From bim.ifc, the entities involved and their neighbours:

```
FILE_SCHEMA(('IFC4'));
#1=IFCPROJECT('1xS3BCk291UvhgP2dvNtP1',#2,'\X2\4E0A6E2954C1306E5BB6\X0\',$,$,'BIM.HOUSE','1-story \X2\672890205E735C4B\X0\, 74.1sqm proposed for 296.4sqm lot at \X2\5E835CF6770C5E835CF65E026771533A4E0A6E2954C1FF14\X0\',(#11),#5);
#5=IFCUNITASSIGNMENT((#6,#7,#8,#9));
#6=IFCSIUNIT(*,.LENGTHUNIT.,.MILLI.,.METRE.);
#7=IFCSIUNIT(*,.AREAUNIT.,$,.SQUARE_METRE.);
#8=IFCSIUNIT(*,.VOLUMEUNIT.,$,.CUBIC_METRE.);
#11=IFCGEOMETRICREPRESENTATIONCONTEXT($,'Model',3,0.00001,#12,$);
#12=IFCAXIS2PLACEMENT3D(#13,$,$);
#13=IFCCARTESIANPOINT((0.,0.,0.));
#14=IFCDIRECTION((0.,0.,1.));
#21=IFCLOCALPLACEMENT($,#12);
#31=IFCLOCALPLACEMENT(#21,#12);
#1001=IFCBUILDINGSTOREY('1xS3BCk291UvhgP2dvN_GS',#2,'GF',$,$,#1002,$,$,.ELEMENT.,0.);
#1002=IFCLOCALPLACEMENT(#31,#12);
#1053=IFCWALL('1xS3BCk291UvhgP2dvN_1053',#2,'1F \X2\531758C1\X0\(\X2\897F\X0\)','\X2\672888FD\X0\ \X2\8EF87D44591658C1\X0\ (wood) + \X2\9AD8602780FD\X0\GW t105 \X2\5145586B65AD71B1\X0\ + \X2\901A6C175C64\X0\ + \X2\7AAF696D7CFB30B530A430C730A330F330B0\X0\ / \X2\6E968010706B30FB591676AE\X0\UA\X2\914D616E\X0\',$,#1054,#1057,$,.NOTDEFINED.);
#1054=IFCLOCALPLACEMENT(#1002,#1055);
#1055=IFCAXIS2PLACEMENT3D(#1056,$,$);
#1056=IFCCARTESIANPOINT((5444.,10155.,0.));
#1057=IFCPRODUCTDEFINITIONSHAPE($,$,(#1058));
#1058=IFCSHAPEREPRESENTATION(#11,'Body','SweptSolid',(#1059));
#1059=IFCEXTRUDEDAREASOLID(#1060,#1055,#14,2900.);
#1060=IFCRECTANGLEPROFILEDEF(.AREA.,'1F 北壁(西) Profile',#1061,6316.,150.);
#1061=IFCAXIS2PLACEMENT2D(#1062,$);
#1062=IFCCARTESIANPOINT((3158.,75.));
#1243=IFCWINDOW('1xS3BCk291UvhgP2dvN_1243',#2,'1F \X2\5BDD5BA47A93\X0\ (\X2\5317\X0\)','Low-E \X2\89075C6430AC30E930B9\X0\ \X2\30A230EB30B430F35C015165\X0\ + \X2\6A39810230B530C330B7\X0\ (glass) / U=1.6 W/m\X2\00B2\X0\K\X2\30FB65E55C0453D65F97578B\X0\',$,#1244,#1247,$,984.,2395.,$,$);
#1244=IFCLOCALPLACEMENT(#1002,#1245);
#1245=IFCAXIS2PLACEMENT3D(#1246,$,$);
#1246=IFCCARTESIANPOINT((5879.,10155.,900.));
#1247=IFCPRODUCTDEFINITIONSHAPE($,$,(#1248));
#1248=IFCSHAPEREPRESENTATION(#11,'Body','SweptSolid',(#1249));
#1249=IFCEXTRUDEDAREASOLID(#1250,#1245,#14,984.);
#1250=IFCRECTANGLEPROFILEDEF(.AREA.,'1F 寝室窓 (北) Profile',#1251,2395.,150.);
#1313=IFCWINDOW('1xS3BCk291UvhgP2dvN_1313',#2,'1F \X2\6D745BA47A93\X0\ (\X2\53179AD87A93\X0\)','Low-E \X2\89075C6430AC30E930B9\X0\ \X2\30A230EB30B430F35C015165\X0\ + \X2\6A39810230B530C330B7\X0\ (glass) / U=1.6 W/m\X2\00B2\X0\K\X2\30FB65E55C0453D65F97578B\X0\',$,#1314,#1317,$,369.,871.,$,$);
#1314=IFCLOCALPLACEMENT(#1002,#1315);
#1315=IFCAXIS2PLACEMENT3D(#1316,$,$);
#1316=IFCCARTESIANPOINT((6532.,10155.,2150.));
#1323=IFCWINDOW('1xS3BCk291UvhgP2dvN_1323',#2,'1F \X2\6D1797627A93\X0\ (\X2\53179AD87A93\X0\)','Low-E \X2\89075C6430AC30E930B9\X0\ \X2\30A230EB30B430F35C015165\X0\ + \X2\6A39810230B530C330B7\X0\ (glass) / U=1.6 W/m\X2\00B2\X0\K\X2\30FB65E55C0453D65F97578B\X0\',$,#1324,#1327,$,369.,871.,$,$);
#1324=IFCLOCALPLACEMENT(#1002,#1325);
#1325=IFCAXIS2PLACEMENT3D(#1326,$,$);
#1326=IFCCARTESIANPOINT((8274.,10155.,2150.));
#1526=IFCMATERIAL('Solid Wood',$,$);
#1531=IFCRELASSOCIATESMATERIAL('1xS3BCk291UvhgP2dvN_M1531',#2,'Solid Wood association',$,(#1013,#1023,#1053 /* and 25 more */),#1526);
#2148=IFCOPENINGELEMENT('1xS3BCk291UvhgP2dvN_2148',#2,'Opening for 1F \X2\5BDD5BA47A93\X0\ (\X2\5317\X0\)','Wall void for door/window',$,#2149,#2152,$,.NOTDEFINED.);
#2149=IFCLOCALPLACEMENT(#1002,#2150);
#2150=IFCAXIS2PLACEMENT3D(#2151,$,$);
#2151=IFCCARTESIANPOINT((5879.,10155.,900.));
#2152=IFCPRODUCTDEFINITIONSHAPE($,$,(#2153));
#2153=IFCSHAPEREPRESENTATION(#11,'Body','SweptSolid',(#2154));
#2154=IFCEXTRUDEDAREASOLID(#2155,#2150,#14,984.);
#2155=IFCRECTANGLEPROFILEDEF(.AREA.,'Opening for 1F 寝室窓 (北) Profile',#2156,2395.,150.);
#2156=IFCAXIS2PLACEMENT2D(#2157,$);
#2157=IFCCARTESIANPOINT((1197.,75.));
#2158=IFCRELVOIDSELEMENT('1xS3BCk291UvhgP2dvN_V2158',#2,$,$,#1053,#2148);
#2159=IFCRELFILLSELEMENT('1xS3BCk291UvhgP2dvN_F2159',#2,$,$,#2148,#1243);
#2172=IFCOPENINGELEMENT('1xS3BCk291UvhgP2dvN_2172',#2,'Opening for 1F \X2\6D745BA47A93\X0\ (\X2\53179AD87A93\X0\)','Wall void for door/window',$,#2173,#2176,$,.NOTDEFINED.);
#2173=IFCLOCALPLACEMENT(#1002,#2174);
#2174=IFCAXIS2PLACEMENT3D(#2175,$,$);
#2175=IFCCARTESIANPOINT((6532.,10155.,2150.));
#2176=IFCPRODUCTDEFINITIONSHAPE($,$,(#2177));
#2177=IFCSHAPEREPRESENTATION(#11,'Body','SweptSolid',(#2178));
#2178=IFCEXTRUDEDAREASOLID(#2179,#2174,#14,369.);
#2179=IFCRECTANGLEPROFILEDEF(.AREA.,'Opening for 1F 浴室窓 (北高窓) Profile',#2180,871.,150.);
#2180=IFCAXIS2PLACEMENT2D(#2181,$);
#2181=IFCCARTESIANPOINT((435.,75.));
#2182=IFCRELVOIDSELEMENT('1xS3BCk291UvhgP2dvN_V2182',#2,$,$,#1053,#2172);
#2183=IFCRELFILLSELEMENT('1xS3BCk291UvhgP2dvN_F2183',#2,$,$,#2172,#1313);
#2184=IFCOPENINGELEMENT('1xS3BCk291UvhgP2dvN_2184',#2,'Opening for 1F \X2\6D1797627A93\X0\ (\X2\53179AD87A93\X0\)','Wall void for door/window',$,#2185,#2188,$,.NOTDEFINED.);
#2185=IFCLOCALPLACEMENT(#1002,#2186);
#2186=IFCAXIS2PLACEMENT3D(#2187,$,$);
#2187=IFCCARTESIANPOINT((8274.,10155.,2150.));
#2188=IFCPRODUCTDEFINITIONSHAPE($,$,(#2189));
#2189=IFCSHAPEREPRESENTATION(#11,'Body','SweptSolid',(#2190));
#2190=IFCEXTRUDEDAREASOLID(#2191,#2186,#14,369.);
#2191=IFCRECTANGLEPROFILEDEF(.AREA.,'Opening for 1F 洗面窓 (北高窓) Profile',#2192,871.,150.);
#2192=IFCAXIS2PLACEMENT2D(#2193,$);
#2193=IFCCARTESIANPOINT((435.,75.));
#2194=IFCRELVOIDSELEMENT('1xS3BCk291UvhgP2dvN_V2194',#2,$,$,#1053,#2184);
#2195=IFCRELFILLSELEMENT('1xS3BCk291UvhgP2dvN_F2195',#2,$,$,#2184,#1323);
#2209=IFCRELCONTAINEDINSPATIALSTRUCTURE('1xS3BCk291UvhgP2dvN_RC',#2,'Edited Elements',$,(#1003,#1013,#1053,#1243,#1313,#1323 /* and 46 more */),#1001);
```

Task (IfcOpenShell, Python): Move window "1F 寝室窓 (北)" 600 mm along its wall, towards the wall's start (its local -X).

```python
import ifcopenshell
import ifcopenshell.api.geometry
import ifcopenshell.util.placement
import ifcopenshell.util.unit

model = ifcopenshell.open("bim.ifc")
unit_scale = ifcopenshell.util.unit.calculate_unit_scale(model)

window = model.by_guid("1xS3BCk291UvhgP2dvN_1243")
opening = window.FillsVoids[0].RelatingOpeningElement
wall = opening.VoidsElements[0].RelatingBuildingElement

wall_matrix = ifcopenshell.util.placement.get_local_placement(wall.ObjectPlacement)
shift = wall_matrix[:3, 0] * -0.6 / unit_scale
before = ifcopenshell.util.placement.get_local_placement(window.ObjectPlacement)[:3, 3].copy()

# The window is not placed relative to its opening, so move both.
for product in (opening, window):
    matrix = ifcopenshell.util.placement.get_local_placement(product.ObjectPlacement)
    matrix[:3, 3] += shift
    ifcopenshell.api.geometry.edit_object_placement(model, product=product, matrix=matrix, is_si=False)

after = ifcopenshell.util.placement.get_local_placement(window.ObjectPlacement)[:3, 3]
print("window moved by", (after - before).round(3) + 0.0)

model.write("bim_rev.ifc")
```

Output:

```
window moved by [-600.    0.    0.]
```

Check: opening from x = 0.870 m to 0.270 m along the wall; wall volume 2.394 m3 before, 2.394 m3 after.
